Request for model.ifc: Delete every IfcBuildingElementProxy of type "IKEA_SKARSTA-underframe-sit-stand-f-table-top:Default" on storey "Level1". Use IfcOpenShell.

First a look at what the model holds.

```python
import ifcopenshell
import ifcopenshell.util.element

model = ifcopenshell.open("model.ifc")
print(model.schema)
storey = next(s for s in model.by_type("IfcBuildingStorey") if s.Name == "Level1")
proxies = [e for e in ifcopenshell.util.element.get_decomposition(storey) if e.is_a("IfcBuildingElementProxy")]
seen = {}
for e in proxies:
    element_type = ifcopenshell.util.element.get_type(e)
    name = element_type.Name if element_type not in (None, e) else None
    seen[name] = seen.get(name, 0) + 1
for name, count in sorted(seen.items(), key=str):
    print(count, "x", name)
```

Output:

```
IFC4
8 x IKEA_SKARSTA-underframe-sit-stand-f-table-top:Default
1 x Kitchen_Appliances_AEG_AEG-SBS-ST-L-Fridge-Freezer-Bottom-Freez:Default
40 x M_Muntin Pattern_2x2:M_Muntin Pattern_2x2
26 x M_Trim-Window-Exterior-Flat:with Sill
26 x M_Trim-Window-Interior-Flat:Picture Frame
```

```python
import ifcopenshell
import ifcopenshell.api.root
import ifcopenshell.util.element

model = ifcopenshell.open("model.ifc")

storey = next(s for s in model.by_type("IfcBuildingStorey") if s.Name == "Level1")
proxies = [e for e in ifcopenshell.util.element.get_decomposition(storey) if e.is_a("IfcBuildingElementProxy")]
targets = [e for e in proxies if (t := ifcopenshell.util.element.get_type(e)) not in (None, e) and t.Name == "IKEA_SKARSTA-underframe-sit-stand-f-table-top:Default"]

for e in targets:
    ifcopenshell.api.root.remove_product(model, product=e)
print(len(targets), "removed")

model.write("model_edited.ifc")
```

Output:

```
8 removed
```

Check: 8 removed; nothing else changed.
